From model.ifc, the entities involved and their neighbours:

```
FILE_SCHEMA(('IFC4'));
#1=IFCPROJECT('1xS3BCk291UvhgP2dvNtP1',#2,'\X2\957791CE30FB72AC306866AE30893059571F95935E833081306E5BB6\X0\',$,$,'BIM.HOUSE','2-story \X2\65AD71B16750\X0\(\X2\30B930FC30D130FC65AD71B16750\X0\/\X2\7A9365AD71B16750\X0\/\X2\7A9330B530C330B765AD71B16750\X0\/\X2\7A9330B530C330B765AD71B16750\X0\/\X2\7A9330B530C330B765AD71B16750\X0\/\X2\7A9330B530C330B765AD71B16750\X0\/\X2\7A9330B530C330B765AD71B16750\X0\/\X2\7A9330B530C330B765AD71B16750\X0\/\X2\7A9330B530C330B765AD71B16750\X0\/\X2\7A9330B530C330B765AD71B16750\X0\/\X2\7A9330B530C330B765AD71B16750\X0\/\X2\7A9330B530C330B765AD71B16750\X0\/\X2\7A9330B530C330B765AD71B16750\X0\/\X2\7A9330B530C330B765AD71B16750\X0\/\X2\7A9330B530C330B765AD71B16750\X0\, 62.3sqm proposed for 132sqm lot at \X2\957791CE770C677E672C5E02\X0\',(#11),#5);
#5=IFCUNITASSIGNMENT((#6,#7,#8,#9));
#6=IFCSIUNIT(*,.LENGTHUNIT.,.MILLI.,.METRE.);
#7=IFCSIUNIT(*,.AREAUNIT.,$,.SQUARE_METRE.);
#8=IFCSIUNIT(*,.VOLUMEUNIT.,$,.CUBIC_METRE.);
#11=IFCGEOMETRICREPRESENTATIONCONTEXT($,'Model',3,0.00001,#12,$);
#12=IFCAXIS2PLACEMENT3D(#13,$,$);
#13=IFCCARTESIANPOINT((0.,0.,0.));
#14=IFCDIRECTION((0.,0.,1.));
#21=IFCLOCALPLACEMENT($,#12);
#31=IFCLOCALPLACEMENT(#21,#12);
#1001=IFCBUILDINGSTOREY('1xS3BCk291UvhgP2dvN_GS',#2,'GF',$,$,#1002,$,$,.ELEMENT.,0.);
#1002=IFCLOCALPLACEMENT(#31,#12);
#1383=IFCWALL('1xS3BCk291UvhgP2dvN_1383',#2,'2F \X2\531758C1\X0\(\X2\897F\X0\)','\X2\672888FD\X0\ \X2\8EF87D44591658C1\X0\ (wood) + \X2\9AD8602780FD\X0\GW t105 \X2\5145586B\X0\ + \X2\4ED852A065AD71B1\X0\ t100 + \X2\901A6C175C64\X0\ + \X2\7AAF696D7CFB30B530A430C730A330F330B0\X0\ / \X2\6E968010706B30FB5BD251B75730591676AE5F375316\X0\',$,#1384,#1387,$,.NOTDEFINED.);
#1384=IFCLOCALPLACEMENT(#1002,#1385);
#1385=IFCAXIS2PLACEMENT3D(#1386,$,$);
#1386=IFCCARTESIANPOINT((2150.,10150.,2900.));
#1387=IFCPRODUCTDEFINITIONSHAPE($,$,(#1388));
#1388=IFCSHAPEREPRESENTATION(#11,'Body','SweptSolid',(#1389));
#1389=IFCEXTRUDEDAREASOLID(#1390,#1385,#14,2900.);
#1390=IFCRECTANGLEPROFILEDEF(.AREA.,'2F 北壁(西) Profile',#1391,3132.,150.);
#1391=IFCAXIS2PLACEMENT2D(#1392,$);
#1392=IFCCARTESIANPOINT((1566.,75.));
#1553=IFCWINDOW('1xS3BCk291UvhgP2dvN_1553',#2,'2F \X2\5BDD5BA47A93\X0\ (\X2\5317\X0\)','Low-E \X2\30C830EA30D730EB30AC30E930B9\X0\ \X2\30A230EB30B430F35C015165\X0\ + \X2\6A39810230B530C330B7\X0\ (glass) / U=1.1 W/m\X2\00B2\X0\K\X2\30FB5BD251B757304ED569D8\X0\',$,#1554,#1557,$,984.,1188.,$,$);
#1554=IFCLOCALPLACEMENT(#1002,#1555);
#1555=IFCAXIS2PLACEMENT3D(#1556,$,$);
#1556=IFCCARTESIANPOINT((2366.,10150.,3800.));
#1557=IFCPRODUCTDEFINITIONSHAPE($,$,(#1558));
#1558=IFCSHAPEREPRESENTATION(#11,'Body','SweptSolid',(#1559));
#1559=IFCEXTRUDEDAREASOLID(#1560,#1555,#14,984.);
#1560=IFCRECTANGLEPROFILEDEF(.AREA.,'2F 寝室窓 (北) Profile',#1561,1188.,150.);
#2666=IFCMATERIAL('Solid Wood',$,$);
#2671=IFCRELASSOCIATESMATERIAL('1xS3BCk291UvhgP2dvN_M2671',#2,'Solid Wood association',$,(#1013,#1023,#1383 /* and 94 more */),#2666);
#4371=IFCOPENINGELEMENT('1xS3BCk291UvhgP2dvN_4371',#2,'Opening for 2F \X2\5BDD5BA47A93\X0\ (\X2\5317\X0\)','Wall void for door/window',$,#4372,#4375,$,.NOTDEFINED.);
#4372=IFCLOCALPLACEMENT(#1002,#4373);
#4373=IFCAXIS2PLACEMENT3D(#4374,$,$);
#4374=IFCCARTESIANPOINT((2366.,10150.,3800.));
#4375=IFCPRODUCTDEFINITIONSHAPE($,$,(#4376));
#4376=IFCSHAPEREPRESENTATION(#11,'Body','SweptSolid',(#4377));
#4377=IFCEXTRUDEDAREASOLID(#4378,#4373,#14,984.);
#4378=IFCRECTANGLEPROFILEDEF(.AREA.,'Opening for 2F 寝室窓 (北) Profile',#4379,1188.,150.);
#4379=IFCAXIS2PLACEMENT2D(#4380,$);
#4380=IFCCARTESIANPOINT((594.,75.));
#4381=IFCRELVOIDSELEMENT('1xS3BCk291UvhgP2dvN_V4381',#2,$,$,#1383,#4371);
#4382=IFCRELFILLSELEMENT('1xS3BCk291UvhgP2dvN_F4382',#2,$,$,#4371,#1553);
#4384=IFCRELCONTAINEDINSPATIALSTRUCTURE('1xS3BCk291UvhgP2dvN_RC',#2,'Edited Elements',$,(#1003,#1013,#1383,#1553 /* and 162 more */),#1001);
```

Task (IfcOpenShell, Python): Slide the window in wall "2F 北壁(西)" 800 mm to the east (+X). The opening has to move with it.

```python
import ifcopenshell
import ifcopenshell.api.geometry
import ifcopenshell.util.placement
import ifcopenshell.util.unit

model = ifcopenshell.open("model.ifc")
unit_scale = ifcopenshell.util.unit.calculate_unit_scale(model)

window = model.by_guid("1xS3BCk291UvhgP2dvN_1553")
opening = window.FillsVoids[0].RelatingOpeningElement
wall = opening.VoidsElements[0].RelatingBuildingElement

wall_matrix = ifcopenshell.util.placement.get_local_placement(wall.ObjectPlacement)
shift = wall_matrix[:3, 0] * 0.8 / unit_scale
before = ifcopenshell.util.placement.get_local_placement(window.ObjectPlacement)[:3, 3].copy()

# The window is not placed relative to its opening, so move both.
for product in (opening, window):
    matrix = ifcopenshell.util.placement.get_local_placement(product.ObjectPlacement)
    matrix[:3, 3] += shift
    ifcopenshell.api.geometry.edit_object_placement(model, product=product, matrix=matrix, is_si=False)

after = ifcopenshell.util.placement.get_local_placement(window.ObjectPlacement)[:3, 3]
print("window moved by", (after - before).round(3) + 0.0)

model.write("model_edited.ifc")
```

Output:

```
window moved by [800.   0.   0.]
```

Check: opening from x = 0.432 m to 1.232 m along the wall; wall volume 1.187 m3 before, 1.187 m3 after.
